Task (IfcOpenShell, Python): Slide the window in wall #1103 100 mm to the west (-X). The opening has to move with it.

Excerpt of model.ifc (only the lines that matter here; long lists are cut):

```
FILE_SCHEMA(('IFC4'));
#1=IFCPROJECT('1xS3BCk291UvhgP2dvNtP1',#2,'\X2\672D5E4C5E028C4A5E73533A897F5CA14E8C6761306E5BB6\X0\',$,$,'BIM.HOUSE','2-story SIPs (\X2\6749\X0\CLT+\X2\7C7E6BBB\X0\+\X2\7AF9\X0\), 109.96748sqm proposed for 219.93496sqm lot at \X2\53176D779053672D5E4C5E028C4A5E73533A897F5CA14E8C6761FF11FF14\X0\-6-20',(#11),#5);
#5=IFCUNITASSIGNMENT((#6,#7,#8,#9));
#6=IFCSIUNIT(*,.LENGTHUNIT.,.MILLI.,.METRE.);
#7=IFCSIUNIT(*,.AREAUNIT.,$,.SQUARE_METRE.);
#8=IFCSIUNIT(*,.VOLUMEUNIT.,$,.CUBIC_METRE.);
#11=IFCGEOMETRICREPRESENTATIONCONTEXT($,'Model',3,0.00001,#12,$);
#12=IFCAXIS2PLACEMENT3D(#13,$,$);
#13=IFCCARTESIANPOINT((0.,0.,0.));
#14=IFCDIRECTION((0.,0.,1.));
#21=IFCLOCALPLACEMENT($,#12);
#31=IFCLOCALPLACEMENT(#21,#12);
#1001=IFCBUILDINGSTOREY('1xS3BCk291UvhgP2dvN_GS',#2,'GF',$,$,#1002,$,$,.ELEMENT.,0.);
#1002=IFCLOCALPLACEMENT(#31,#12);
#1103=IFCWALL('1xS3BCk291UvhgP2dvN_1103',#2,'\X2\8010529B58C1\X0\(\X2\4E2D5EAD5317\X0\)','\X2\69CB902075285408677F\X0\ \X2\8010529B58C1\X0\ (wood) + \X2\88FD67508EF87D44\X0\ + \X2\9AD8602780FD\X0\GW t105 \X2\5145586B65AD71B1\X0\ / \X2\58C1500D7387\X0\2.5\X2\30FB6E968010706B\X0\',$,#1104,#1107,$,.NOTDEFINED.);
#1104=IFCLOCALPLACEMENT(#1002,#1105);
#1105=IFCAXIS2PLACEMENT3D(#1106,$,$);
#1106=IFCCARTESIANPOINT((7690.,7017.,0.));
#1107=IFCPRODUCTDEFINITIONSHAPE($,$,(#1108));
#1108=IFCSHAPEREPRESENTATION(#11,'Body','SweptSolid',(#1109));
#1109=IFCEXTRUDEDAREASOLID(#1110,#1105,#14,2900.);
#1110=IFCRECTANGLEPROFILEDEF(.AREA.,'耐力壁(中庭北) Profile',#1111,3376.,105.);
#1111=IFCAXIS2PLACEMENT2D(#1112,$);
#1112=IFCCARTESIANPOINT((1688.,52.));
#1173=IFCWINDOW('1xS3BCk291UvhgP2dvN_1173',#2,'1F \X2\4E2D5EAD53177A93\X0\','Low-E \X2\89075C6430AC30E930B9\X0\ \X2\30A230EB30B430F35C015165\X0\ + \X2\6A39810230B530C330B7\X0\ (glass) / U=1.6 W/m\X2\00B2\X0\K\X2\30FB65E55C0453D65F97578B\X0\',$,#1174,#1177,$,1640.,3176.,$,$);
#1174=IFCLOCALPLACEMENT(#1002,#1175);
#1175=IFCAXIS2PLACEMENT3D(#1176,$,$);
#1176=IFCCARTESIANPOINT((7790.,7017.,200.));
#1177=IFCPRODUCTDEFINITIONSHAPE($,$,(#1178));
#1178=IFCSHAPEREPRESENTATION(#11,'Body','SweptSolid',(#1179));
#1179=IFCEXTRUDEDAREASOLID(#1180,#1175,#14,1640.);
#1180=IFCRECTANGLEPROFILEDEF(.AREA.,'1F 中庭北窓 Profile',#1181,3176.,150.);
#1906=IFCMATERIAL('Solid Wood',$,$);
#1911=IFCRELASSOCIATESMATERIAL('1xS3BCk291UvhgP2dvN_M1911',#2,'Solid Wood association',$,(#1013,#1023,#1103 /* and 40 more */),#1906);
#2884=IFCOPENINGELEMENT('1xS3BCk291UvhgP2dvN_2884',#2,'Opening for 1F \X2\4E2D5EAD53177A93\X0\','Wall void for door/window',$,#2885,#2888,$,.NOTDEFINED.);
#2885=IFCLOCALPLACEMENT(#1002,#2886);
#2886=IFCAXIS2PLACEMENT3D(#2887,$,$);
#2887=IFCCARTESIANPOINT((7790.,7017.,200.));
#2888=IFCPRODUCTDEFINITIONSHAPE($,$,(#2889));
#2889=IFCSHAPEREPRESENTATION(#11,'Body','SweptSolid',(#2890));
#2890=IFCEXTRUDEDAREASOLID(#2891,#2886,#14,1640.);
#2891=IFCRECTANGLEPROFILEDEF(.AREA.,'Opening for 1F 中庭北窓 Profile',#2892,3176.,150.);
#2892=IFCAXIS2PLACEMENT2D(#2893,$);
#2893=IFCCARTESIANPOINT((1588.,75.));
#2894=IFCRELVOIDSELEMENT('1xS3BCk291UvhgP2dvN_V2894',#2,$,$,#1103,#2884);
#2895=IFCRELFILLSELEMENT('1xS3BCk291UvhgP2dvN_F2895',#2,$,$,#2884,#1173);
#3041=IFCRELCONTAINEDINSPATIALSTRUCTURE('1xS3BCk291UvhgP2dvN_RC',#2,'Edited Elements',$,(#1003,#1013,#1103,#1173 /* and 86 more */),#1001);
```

```python
import ifcopenshell
import ifcopenshell.api.geometry
import ifcopenshell.util.placement
import ifcopenshell.util.unit

model = ifcopenshell.open("model.ifc")
unit_scale = ifcopenshell.util.unit.calculate_unit_scale(model)

window = model.by_guid("1xS3BCk291UvhgP2dvN_1173")
opening = window.FillsVoids[0].RelatingOpeningElement
wall = opening.VoidsElements[0].RelatingBuildingElement

wall_matrix = ifcopenshell.util.placement.get_local_placement(wall.ObjectPlacement)
shift = wall_matrix[:3, 0] * -0.1 / unit_scale
before = ifcopenshell.util.placement.get_local_placement(window.ObjectPlacement)[:3, 3].copy()

# The window is not placed relative to its opening, so move both.
for product in (opening, window):
    matrix = ifcopenshell.util.placement.get_local_placement(product.ObjectPlacement)
    matrix[:3, 3] += shift
    ifcopenshell.api.geometry.edit_object_placement(model, product=product, matrix=matrix, is_si=False)

after = ifcopenshell.util.placement.get_local_placement(window.ObjectPlacement)[:3, 3]
print("window moved by", (after - before).round(3) + 0.0)

model.write("model_updated.ifc")
```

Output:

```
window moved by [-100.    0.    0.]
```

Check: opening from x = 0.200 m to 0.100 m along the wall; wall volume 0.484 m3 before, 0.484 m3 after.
